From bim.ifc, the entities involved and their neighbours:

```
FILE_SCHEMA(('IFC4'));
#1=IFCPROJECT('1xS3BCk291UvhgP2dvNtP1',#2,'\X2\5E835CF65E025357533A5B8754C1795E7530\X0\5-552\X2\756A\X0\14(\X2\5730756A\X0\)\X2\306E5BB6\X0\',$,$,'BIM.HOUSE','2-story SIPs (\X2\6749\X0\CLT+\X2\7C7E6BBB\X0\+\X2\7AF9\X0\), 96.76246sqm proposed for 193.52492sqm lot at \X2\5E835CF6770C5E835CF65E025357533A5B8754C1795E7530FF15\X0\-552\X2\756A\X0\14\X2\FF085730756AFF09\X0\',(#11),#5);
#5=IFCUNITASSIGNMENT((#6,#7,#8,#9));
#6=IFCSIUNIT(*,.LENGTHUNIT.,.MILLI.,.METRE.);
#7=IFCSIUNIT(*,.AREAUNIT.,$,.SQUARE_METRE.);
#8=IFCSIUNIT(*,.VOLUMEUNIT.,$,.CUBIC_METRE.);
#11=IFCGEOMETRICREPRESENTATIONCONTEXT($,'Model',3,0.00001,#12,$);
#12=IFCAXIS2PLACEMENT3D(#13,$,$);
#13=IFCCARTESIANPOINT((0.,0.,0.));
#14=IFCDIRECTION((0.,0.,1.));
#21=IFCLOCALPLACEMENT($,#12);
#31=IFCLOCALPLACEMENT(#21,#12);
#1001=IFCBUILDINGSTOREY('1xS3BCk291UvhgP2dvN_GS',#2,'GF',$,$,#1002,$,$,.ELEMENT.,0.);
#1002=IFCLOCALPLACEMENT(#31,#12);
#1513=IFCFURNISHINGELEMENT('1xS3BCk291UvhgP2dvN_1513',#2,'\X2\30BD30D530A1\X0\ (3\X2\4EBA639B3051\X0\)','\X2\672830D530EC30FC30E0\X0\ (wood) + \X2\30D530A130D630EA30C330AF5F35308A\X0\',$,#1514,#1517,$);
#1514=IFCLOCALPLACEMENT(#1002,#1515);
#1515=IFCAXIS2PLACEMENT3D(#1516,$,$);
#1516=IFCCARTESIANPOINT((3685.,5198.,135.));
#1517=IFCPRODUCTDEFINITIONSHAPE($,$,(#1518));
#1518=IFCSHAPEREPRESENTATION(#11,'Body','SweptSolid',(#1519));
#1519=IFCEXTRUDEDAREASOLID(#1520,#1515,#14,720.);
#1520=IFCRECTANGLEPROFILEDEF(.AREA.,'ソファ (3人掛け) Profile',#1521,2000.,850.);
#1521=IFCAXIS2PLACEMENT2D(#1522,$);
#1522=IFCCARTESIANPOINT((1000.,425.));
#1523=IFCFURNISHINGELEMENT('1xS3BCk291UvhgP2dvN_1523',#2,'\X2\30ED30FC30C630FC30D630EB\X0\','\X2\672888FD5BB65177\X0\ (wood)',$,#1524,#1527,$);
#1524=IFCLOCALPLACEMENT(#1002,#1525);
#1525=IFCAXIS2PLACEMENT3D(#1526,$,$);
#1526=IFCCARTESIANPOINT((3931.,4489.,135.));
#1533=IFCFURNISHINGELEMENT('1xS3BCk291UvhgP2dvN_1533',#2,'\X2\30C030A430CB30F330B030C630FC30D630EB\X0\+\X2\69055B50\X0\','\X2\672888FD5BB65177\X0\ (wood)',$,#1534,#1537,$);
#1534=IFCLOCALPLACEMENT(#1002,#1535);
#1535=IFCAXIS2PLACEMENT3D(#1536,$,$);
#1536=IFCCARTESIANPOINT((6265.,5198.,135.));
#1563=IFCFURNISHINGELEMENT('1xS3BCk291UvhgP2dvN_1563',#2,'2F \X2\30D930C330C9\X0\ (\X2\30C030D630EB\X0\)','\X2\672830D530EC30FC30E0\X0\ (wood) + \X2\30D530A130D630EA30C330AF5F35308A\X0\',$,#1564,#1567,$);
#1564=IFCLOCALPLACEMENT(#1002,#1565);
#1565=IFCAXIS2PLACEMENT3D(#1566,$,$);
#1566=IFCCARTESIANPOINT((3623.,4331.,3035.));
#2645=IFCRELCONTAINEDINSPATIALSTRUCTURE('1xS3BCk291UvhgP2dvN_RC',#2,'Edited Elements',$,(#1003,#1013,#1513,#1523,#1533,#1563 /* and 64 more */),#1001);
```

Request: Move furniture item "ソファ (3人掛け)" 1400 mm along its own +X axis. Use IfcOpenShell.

```python
import ifcopenshell
import ifcopenshell.api.geometry
import ifcopenshell.util.placement

model = ifcopenshell.open("bim.ifc")

item = model.by_guid("1xS3BCk291UvhgP2dvN_1513")
matrix = ifcopenshell.util.placement.get_local_placement(item.ObjectPlacement)
matrix[:3, 3] += matrix[:3, 0] * 1400.0
ifcopenshell.api.geometry.edit_object_placement(model, product=item, matrix=matrix, is_si=False)

print(ifcopenshell.util.placement.get_local_placement(item.ObjectPlacement).round(3) + 0.0)

model.write("bim_updated.ifc")
```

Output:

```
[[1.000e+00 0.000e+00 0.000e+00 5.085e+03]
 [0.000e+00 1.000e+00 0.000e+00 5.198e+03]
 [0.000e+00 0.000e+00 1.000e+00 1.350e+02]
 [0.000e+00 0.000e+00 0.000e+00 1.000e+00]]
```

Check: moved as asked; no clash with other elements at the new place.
